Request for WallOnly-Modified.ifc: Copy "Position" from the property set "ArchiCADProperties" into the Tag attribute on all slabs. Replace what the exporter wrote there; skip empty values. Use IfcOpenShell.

First a look at what the model holds.

```python
import ifcopenshell
import ifcopenshell.util.element

model = ifcopenshell.open("WallOnly-Modified.ifc")
print(model.schema)
slabs = model.by_type("IfcSlab")
print(len(slabs), "slabs")
for e in slabs[:8]:
    source = ifcopenshell.util.element.get_pset(e, "ArchiCADProperties", "Position")
    target = e.Tag
    print(e.id(), repr(source), repr(target), sep=" | ")
```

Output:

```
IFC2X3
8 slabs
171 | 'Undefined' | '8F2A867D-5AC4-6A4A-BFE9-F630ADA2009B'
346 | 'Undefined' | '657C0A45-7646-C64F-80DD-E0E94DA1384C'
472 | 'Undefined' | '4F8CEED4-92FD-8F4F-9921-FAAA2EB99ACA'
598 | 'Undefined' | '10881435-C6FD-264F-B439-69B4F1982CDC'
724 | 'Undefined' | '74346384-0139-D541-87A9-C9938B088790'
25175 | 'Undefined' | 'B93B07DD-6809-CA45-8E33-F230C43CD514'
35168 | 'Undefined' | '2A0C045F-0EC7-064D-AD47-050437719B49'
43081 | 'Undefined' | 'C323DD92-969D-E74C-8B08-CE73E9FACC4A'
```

```python
import ifcopenshell
import ifcopenshell.util.element

model = ifcopenshell.open("WallOnly-Modified.ifc")

count = 0
for e in model.by_type("IfcSlab"):
    value = ifcopenshell.util.element.get_pset(e, "ArchiCADProperties", "Position")
    current = e.Tag
    if not value or not value.strip() or current == value:
        continue
    e.Tag = value
    count += 1

print(count, "slabs updated")

model.write("WallOnly-Modified-out.ifc")
```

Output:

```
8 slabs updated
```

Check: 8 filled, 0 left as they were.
